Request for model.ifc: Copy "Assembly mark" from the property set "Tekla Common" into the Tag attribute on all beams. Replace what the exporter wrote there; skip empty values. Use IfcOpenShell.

First a look at what the model holds.

```python
import ifcopenshell
import ifcopenshell.util.element

model = ifcopenshell.open("model.ifc")
print(model.schema)
beams = model.by_type("IfcBeam")
print(len(beams), "beams")
for e in beams[:8]:
    source = ifcopenshell.util.element.get_pset(e, "Tekla Common", "Assembly mark")
    target = e.Tag
    print(e.id(), repr(source), repr(target), sep=" | ")
```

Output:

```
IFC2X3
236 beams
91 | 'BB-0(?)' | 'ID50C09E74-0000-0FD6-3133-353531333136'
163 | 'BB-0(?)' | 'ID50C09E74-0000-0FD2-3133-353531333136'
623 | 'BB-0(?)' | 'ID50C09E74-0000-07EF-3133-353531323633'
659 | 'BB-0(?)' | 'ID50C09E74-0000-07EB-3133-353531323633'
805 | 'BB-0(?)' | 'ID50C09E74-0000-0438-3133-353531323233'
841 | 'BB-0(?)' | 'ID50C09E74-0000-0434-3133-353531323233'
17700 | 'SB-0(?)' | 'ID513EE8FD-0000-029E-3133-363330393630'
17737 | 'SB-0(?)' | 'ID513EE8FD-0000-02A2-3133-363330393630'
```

```python
import ifcopenshell
import ifcopenshell.util.element

model = ifcopenshell.open("model.ifc")

count = 0
for e in model.by_type("IfcBeam"):
    value = ifcopenshell.util.element.get_pset(e, "Tekla Common", "Assembly mark")
    current = e.Tag
    if not value or not value.strip() or current == value:
        continue
    e.Tag = value
    count += 1

print(count, "beams updated")

model.write("model_updated.ifc")
```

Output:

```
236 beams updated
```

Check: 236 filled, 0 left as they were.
